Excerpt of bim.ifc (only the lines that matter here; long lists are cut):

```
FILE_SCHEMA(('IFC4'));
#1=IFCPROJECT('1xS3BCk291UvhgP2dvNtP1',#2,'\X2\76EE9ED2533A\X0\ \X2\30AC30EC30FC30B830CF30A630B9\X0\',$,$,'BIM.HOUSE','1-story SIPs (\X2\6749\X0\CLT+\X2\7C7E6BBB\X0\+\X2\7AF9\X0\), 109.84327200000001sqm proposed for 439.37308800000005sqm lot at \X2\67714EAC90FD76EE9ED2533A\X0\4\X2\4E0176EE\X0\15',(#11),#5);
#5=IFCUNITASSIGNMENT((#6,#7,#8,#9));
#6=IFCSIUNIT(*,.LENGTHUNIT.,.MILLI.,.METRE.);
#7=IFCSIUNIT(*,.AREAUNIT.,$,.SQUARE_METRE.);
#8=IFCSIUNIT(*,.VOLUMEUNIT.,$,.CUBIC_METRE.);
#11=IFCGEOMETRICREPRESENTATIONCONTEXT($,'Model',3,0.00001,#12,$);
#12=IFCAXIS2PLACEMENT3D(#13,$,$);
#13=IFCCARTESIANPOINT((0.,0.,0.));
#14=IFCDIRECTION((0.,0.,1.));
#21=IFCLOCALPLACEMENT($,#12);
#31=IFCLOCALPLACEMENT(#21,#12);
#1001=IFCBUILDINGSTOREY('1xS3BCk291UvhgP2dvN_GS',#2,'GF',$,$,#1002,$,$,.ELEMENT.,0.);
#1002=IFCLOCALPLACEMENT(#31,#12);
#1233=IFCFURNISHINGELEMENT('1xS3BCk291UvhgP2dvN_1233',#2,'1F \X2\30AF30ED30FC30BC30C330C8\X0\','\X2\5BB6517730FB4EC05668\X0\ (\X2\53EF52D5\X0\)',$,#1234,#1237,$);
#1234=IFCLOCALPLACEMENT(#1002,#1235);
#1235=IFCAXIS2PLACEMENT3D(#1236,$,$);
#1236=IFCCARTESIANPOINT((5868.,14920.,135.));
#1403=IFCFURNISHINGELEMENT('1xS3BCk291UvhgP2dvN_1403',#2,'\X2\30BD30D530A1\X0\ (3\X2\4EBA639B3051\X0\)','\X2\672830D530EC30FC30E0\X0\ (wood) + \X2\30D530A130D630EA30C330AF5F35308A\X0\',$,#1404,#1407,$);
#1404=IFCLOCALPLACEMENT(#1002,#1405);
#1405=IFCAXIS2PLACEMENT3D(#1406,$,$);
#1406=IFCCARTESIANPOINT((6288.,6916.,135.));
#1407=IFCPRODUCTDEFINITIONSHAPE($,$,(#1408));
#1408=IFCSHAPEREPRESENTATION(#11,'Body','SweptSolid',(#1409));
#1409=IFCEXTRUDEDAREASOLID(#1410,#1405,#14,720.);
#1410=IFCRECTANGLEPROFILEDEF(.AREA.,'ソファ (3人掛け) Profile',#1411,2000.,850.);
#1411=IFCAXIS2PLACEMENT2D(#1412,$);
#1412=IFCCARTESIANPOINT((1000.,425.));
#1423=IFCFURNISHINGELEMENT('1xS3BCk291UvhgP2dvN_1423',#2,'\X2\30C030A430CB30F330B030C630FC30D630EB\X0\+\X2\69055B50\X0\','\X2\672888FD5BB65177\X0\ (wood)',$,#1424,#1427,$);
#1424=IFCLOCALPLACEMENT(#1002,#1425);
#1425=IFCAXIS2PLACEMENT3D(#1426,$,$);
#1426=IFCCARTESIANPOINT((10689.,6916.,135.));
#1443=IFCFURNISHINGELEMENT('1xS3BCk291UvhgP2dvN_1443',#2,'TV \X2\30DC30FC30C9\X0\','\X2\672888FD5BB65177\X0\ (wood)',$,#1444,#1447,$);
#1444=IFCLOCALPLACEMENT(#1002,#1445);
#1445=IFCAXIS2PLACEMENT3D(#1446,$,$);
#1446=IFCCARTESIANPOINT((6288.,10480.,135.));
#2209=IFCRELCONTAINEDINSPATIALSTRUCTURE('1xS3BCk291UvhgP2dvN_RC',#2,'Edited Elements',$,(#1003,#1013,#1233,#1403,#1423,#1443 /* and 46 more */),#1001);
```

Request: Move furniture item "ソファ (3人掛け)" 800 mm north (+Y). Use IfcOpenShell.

```python
import ifcopenshell
import ifcopenshell.api.geometry
import ifcopenshell.util.placement
import ifcopenshell.util.unit

model = ifcopenshell.open("bim.ifc")
unit_scale = ifcopenshell.util.unit.calculate_unit_scale(model)

item = model.by_guid("1xS3BCk291UvhgP2dvN_1403")
matrix = ifcopenshell.util.placement.get_local_placement(item.ObjectPlacement)
matrix[1, 3] += 0.8 / unit_scale
ifcopenshell.api.geometry.edit_object_placement(model, product=item, matrix=matrix, is_si=False)

print(ifcopenshell.util.placement.get_local_placement(item.ObjectPlacement).round(3) + 0.0)

model.write("bim_v2.ifc")
```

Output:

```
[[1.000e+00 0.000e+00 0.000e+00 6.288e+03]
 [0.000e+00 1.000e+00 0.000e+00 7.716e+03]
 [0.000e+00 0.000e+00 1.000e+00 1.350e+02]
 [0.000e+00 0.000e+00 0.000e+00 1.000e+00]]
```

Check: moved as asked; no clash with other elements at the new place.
